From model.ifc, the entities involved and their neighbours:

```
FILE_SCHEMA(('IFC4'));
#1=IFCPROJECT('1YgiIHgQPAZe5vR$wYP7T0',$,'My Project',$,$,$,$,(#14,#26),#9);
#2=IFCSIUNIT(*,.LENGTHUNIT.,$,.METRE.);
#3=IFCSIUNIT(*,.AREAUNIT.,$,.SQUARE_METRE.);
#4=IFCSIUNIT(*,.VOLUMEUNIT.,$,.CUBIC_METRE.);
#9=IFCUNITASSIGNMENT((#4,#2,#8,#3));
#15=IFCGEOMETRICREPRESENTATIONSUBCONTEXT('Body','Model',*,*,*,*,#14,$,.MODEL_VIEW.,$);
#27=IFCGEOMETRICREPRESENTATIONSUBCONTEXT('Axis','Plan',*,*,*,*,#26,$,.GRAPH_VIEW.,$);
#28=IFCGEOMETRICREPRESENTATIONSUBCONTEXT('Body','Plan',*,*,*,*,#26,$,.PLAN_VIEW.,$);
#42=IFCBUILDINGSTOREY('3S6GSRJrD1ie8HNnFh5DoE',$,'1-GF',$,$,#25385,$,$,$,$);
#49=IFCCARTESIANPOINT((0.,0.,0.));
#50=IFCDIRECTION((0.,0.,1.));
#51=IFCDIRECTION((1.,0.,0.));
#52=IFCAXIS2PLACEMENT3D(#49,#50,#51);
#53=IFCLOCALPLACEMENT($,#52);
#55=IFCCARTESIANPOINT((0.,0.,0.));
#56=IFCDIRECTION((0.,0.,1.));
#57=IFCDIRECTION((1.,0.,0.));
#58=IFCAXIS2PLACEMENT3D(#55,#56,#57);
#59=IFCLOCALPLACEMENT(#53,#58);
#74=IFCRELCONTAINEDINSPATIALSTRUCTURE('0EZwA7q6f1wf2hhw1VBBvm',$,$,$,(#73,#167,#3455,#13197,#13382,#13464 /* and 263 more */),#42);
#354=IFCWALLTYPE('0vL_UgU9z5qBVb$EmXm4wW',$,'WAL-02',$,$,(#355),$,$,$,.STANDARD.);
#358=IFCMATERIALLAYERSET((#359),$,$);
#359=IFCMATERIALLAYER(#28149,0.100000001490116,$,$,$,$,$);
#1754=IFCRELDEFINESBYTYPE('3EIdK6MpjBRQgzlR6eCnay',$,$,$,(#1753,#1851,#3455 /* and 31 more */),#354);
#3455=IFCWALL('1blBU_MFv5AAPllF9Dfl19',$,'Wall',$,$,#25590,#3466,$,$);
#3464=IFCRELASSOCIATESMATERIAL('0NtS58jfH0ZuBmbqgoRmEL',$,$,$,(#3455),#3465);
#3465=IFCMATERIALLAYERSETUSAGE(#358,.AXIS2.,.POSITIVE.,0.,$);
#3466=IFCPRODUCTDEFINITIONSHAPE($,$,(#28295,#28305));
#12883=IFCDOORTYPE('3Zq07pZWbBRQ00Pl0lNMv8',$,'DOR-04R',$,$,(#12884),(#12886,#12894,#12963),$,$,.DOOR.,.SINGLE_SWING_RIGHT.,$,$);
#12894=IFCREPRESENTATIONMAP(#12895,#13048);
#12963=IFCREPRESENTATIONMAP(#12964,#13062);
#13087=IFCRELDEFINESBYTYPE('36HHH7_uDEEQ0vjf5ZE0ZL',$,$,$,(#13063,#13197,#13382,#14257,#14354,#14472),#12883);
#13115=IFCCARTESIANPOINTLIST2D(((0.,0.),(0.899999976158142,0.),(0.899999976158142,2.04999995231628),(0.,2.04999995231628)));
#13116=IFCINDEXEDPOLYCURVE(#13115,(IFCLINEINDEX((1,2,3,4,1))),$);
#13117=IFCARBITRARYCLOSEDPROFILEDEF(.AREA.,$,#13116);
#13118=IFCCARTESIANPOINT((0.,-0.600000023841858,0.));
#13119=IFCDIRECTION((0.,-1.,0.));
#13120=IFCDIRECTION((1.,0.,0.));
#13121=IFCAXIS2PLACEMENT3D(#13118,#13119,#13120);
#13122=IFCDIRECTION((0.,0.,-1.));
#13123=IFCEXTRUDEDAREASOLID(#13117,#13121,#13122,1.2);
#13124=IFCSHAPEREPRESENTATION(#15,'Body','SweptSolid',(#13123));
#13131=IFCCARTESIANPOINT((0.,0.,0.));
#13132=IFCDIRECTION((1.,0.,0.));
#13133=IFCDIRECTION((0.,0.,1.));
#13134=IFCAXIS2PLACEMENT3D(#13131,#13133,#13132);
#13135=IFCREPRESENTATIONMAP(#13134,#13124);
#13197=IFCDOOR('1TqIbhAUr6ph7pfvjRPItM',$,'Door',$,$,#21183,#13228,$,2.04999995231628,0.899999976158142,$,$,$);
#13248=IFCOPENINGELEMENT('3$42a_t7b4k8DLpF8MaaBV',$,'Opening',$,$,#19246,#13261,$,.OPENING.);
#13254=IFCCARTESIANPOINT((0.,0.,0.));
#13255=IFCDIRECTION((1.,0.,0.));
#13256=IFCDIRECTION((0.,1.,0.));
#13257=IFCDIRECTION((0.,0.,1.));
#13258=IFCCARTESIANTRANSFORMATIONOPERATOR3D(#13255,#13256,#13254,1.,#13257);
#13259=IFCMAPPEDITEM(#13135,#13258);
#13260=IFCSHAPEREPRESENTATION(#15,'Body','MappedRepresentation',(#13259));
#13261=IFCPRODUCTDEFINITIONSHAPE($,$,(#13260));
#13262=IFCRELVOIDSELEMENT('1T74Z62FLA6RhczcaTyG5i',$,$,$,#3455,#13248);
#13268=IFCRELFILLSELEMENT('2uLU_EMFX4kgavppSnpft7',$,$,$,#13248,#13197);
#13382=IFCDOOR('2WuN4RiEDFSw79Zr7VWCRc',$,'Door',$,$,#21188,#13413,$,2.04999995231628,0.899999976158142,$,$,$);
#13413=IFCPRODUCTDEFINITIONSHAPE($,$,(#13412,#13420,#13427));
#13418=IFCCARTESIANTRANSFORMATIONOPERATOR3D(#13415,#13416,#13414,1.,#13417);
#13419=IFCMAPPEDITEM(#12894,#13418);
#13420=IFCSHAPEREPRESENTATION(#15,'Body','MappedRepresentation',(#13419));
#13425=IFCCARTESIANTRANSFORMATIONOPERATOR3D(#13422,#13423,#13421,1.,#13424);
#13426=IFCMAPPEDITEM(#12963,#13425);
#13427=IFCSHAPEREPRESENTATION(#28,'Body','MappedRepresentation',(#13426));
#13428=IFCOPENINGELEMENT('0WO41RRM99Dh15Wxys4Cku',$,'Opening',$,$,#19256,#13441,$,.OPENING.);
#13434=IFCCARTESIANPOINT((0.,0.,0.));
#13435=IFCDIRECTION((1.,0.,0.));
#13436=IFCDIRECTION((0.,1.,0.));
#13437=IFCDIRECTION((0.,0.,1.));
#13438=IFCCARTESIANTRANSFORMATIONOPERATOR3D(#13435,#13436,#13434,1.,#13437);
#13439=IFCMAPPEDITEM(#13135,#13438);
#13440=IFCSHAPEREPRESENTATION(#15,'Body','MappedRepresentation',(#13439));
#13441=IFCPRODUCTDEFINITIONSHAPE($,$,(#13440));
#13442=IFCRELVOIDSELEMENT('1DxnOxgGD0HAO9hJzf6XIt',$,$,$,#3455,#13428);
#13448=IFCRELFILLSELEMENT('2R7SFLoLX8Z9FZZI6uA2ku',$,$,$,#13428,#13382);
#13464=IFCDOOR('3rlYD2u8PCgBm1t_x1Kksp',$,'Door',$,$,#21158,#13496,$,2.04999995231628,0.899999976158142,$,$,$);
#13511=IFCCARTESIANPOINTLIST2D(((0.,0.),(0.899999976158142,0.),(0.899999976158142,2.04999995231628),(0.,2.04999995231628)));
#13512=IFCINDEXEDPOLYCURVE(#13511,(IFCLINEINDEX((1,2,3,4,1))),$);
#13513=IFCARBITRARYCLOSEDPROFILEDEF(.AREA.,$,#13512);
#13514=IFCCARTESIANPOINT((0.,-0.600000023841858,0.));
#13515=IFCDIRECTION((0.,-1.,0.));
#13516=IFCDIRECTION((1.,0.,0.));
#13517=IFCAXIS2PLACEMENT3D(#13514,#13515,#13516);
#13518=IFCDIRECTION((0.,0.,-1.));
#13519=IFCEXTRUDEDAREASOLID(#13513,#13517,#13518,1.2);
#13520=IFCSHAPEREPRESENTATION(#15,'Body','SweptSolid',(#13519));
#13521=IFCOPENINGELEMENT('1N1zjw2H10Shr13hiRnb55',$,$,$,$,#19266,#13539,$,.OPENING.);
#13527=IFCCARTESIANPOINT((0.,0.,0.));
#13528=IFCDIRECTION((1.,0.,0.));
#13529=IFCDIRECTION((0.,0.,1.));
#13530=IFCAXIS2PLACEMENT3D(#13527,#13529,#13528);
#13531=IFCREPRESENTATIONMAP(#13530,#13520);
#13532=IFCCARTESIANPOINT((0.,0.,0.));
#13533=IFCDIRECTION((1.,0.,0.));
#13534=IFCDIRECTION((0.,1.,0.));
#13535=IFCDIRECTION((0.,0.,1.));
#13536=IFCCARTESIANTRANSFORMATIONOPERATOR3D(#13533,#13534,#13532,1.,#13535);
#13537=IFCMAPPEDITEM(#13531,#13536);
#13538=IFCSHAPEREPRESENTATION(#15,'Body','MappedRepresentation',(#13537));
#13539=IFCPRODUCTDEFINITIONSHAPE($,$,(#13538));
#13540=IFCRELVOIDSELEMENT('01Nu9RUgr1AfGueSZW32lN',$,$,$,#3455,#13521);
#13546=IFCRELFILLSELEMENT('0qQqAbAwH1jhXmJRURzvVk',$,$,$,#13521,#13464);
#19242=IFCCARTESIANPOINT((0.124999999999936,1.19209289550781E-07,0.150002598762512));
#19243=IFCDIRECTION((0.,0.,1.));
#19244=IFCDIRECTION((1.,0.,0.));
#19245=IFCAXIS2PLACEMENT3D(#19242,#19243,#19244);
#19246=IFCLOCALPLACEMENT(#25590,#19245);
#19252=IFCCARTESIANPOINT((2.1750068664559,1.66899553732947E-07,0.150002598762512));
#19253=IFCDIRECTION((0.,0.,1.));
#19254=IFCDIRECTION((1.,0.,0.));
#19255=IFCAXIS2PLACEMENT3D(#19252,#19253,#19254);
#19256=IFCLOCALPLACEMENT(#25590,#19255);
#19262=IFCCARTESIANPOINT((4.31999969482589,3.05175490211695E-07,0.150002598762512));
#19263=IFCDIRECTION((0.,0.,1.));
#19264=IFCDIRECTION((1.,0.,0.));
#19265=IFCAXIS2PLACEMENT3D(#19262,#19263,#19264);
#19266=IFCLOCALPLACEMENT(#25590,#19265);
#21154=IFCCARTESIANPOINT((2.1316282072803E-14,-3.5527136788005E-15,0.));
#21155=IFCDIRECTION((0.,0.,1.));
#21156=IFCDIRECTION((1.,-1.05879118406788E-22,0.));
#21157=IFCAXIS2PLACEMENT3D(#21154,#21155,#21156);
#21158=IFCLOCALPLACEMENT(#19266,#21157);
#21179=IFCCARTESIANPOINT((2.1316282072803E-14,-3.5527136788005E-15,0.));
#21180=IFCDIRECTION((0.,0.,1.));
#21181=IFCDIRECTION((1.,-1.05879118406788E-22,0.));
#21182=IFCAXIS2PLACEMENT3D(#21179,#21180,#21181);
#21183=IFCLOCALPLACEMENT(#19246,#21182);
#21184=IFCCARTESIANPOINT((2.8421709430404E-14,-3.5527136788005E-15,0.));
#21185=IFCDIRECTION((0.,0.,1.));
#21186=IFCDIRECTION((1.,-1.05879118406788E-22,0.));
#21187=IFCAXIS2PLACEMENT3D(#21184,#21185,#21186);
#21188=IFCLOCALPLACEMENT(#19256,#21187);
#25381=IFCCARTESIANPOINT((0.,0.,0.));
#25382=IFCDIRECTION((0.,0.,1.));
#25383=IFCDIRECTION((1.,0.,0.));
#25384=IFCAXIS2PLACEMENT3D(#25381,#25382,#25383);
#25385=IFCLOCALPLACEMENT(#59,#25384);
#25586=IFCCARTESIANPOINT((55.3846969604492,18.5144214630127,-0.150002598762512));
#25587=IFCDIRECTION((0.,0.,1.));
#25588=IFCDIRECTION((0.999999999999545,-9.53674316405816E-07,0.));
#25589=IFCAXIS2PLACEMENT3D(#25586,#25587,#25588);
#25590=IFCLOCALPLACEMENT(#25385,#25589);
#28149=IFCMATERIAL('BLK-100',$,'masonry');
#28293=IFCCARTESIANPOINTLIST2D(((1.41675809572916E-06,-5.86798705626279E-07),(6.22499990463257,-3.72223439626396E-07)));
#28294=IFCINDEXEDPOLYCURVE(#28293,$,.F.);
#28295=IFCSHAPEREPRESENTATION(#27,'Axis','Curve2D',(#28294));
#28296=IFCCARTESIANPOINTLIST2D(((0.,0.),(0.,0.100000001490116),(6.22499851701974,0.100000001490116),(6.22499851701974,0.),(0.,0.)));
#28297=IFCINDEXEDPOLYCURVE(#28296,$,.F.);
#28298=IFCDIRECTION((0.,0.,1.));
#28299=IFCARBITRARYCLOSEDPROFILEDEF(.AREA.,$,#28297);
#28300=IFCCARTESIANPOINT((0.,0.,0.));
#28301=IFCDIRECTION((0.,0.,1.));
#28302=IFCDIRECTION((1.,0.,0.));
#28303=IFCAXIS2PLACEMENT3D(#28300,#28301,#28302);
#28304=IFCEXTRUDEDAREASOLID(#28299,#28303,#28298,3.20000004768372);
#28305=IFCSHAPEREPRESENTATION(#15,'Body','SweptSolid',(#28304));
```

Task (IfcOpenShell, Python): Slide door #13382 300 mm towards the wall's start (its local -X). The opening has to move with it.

```python
import ifcopenshell
import ifcopenshell.api.geometry
import ifcopenshell.util.placement
import ifcopenshell.util.unit

model = ifcopenshell.open("model.ifc")
unit_scale = ifcopenshell.util.unit.calculate_unit_scale(model)

door = model.by_guid("2WuN4RiEDFSw79Zr7VWCRc")
opening = door.FillsVoids[0].RelatingOpeningElement
wall = opening.VoidsElements[0].RelatingBuildingElement

wall_matrix = ifcopenshell.util.placement.get_local_placement(wall.ObjectPlacement)
shift = wall_matrix[:3, 0] * -0.3 / unit_scale
before = ifcopenshell.util.placement.get_local_placement(door.ObjectPlacement)[:3, 3].copy()

# The door is placed relative to its opening, so it follows when the opening moves.
matrix = ifcopenshell.util.placement.get_local_placement(opening.ObjectPlacement)
matrix[:3, 3] += shift
ifcopenshell.api.geometry.edit_object_placement(
    model, product=opening, matrix=matrix, is_si=False, should_transform_children=True
)

after = ifcopenshell.util.placement.get_local_placement(door.ObjectPlacement)[:3, 3]
print("door moved by", (after - before).round(3) + 0.0)

model.write("model-out.ifc")
```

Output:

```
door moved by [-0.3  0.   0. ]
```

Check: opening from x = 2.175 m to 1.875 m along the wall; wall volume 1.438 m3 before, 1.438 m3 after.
